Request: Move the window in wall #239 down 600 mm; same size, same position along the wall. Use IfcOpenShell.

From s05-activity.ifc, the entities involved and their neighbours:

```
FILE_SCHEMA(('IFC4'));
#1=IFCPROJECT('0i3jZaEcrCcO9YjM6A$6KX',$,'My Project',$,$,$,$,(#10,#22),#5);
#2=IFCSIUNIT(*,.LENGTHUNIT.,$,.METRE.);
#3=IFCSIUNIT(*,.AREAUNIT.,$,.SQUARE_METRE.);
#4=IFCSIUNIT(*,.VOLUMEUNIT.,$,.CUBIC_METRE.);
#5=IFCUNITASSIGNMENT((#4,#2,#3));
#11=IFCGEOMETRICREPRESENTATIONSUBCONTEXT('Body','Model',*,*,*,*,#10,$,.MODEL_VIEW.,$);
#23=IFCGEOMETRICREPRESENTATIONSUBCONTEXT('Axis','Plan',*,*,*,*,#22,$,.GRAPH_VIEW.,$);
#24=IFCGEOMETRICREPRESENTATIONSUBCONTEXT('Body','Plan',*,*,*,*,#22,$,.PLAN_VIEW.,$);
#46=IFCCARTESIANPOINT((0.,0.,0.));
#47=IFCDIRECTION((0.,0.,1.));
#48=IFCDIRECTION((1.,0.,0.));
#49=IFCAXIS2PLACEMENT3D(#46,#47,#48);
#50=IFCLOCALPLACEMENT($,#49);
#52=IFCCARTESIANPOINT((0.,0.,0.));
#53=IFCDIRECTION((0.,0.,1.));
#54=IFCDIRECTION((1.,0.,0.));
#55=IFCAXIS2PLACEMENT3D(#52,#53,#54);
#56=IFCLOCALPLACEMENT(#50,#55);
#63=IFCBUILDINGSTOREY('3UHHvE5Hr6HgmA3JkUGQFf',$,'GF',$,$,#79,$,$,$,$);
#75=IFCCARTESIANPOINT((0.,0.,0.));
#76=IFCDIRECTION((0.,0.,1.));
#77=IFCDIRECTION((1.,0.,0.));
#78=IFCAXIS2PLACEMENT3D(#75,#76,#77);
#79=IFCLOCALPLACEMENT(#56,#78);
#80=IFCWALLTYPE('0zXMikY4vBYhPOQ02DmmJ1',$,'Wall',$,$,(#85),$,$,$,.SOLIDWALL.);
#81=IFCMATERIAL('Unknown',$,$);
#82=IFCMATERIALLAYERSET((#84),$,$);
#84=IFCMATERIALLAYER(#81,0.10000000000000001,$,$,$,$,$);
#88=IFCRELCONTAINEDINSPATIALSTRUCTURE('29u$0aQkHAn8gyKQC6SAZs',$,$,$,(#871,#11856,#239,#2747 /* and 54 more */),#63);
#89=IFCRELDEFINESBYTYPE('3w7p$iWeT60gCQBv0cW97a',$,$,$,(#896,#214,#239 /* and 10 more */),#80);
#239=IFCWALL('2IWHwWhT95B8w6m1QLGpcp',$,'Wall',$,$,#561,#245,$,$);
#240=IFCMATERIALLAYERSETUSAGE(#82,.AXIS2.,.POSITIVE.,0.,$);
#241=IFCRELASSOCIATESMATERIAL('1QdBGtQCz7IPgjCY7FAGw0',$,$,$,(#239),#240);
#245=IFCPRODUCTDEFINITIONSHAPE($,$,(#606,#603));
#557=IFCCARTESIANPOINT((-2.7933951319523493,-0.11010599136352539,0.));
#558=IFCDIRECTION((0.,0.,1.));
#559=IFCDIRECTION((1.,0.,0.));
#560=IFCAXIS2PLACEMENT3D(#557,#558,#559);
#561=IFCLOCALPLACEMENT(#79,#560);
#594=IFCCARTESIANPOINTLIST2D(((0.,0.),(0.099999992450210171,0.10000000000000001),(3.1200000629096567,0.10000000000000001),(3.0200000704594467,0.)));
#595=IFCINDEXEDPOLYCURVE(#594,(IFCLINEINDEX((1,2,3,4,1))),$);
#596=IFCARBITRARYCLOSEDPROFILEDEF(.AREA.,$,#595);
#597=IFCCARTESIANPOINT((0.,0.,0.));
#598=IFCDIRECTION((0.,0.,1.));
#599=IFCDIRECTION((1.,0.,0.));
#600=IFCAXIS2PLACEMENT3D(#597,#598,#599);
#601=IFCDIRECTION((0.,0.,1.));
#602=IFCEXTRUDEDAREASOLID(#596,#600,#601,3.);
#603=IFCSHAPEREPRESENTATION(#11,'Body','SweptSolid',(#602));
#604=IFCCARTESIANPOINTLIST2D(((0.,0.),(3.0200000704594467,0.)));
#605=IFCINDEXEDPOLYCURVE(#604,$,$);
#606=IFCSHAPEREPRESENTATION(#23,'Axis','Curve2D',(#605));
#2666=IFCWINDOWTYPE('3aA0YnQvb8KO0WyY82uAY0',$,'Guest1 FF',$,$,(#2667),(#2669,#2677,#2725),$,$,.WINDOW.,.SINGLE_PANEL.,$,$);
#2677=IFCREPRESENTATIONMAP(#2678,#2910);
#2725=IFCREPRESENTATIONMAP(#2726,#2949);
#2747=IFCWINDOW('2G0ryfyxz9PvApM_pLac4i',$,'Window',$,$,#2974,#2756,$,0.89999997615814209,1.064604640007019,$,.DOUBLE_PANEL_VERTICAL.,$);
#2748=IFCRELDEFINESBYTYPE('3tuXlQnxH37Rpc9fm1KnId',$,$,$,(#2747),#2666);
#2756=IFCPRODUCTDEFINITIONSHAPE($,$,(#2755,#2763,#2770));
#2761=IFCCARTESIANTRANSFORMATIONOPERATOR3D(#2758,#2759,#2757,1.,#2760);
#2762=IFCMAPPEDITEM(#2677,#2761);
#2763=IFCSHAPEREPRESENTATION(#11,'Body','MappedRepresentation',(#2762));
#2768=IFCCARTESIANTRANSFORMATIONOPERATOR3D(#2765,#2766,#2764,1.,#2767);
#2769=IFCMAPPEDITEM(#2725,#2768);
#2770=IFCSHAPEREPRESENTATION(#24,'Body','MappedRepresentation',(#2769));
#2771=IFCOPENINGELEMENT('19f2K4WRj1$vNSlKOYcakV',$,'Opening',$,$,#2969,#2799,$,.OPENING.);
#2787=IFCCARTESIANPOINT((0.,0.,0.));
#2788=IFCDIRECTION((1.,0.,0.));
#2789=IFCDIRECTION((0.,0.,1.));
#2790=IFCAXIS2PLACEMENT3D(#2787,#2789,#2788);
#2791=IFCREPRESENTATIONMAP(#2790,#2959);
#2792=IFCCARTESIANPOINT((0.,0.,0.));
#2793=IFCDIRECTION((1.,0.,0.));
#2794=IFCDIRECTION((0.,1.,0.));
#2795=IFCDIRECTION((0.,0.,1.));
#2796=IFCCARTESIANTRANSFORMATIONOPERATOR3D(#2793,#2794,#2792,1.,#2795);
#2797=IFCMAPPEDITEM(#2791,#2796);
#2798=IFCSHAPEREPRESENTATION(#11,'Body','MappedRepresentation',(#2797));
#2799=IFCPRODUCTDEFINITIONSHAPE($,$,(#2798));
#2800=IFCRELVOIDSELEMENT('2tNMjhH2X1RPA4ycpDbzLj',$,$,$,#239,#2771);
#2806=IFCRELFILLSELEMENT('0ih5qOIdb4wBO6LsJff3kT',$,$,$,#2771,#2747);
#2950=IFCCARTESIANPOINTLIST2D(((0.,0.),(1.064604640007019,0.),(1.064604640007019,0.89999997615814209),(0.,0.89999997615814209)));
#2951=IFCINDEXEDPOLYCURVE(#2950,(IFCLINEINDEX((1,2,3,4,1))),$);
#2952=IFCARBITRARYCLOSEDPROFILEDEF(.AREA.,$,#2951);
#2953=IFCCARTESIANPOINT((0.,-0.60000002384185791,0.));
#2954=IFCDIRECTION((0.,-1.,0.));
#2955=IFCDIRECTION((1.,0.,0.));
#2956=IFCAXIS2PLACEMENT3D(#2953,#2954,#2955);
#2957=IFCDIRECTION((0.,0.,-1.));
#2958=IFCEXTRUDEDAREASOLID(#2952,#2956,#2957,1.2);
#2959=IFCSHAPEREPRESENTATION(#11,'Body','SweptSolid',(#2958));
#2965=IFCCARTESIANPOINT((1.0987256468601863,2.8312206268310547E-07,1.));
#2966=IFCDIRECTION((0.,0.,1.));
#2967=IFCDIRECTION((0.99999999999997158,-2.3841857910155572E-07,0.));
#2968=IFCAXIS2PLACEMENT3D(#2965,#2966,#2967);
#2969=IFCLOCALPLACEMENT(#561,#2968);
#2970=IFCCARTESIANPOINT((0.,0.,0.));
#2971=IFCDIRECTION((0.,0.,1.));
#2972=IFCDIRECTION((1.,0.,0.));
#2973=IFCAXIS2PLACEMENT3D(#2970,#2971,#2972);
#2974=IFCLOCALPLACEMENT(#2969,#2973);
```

```python
import numpy as np
import ifcopenshell
import ifcopenshell.api.geometry
import ifcopenshell.util.placement
import ifcopenshell.util.unit

model = ifcopenshell.open("s05-activity.ifc")
unit_scale = ifcopenshell.util.unit.calculate_unit_scale(model)

window = model.by_guid("2G0ryfyxz9PvApM_pLac4i")
opening = window.FillsVoids[0].RelatingOpeningElement
dz = -0.6 / unit_scale

shift = np.array([0.0, 0.0, dz])
# The window is placed relative to its opening, so it follows when the opening moves.
matrix = ifcopenshell.util.placement.get_local_placement(opening.ObjectPlacement)
matrix[:3, 3] += shift
ifcopenshell.api.geometry.edit_object_placement(
    model, product=opening, matrix=matrix, is_si=False, should_transform_children=True
)

print(f"moved by {dz * unit_scale:+.3f} m")

model.write("s05-activity_edited.ifc")
```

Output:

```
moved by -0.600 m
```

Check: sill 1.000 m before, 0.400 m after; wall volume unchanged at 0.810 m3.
